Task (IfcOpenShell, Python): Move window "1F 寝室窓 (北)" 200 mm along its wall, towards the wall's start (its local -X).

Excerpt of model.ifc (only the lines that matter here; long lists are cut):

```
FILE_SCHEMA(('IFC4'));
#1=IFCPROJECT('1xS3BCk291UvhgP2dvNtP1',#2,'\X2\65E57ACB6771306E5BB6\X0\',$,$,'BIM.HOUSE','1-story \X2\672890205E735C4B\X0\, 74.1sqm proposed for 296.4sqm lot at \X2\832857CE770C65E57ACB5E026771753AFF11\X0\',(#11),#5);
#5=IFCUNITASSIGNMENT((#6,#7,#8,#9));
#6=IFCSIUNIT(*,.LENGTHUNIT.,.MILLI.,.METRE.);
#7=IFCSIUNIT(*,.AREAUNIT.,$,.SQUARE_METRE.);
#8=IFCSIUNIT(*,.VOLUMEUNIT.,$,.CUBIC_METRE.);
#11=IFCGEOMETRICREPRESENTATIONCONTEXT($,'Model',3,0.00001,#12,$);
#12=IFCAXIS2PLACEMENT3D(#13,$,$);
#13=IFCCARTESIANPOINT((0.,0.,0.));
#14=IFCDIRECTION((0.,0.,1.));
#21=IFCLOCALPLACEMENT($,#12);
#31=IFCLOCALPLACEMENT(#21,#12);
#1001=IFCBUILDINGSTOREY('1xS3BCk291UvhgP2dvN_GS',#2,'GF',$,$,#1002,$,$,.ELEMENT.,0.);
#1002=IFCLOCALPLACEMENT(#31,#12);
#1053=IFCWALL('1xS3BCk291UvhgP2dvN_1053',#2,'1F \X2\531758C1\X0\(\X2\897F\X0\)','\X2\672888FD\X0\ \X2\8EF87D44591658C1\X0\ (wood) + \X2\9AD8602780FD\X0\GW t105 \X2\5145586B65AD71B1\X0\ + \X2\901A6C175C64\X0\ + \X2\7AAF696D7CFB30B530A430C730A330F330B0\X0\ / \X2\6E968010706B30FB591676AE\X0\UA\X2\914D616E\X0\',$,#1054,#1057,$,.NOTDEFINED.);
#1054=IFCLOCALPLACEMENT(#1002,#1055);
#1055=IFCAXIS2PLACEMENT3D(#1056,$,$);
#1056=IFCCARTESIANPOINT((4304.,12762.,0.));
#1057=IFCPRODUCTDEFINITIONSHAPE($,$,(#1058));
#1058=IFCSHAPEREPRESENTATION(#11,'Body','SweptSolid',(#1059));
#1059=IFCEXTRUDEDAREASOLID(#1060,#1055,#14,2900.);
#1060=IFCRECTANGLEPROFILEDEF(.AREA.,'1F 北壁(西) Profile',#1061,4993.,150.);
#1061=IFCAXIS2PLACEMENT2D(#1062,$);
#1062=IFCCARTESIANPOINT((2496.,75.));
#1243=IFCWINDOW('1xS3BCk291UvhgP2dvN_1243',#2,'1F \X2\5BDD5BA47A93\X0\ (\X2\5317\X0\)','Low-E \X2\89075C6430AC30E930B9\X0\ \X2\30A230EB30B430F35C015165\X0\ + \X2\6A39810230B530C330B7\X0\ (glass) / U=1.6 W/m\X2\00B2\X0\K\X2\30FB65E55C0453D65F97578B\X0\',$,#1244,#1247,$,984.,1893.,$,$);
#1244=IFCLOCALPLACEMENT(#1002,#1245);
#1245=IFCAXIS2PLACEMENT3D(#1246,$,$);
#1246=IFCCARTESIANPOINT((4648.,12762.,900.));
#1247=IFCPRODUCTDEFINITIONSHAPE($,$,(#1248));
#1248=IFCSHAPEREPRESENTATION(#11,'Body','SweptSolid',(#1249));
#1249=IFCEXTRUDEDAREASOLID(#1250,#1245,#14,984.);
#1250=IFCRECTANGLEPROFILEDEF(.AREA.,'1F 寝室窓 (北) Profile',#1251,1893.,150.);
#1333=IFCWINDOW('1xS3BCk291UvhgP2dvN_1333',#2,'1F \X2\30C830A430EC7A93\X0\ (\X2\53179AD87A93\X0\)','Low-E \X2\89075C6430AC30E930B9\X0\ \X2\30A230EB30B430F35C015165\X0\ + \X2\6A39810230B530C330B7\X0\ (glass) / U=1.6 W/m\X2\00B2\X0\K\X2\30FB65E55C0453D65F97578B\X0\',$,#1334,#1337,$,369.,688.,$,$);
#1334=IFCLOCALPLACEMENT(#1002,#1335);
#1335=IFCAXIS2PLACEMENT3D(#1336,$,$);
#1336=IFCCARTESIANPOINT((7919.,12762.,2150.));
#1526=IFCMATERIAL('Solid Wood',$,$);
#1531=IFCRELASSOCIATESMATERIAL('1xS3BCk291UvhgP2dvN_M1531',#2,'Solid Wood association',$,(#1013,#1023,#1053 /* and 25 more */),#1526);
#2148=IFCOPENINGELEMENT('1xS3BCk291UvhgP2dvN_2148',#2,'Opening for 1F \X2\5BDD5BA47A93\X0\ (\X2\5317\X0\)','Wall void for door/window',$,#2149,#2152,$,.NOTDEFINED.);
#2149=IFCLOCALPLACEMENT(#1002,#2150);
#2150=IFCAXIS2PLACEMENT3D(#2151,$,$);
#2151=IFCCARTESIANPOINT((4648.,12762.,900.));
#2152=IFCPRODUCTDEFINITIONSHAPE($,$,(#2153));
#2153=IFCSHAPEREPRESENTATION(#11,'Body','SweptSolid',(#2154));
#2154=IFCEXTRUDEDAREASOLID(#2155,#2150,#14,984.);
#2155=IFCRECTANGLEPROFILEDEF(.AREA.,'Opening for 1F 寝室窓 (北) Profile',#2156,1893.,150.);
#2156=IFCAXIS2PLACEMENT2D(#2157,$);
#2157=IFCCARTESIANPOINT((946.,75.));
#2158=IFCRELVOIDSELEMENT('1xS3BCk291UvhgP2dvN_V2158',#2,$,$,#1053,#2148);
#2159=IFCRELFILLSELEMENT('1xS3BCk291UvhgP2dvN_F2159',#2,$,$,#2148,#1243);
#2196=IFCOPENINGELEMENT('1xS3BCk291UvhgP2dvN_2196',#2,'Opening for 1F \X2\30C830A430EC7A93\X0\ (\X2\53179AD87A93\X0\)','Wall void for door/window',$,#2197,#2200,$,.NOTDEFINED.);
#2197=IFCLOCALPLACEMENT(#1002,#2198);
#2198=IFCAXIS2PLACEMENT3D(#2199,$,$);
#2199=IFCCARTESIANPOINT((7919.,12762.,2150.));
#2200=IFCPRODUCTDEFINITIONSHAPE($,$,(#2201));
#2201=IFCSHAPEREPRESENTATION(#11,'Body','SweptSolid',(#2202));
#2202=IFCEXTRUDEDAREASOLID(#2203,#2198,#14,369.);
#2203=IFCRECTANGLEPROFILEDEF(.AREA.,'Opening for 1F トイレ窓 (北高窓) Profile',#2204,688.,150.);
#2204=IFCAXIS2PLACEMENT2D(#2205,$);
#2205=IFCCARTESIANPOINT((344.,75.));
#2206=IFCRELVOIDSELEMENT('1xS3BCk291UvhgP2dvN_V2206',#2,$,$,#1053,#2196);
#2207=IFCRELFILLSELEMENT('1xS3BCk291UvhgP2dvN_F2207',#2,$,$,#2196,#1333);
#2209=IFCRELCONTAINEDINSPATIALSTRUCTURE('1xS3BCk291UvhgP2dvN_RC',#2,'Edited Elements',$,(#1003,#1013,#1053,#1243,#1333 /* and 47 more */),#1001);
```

```python
import ifcopenshell
import ifcopenshell.api.geometry
import ifcopenshell.util.placement

model = ifcopenshell.open("model.ifc")

window = model.by_guid("1xS3BCk291UvhgP2dvN_1243")
opening = window.FillsVoids[0].RelatingOpeningElement
wall = opening.VoidsElements[0].RelatingBuildingElement

wall_matrix = ifcopenshell.util.placement.get_local_placement(wall.ObjectPlacement)
shift = wall_matrix[:3, 0] * -200.0
before = ifcopenshell.util.placement.get_local_placement(window.ObjectPlacement)[:3, 3].copy()

# The window is not placed relative to its opening, so move both.
for product in (opening, window):
    matrix = ifcopenshell.util.placement.get_local_placement(product.ObjectPlacement)
    matrix[:3, 3] += shift
    ifcopenshell.api.geometry.edit_object_placement(model, product=product, matrix=matrix, is_si=False)

after = ifcopenshell.util.placement.get_local_placement(window.ObjectPlacement)[:3, 3]
print("window moved by", (after - before).round(3) + 0.0)

model.write("model_edited.ifc")
```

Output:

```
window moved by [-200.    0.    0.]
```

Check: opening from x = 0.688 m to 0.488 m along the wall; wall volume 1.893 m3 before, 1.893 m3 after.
